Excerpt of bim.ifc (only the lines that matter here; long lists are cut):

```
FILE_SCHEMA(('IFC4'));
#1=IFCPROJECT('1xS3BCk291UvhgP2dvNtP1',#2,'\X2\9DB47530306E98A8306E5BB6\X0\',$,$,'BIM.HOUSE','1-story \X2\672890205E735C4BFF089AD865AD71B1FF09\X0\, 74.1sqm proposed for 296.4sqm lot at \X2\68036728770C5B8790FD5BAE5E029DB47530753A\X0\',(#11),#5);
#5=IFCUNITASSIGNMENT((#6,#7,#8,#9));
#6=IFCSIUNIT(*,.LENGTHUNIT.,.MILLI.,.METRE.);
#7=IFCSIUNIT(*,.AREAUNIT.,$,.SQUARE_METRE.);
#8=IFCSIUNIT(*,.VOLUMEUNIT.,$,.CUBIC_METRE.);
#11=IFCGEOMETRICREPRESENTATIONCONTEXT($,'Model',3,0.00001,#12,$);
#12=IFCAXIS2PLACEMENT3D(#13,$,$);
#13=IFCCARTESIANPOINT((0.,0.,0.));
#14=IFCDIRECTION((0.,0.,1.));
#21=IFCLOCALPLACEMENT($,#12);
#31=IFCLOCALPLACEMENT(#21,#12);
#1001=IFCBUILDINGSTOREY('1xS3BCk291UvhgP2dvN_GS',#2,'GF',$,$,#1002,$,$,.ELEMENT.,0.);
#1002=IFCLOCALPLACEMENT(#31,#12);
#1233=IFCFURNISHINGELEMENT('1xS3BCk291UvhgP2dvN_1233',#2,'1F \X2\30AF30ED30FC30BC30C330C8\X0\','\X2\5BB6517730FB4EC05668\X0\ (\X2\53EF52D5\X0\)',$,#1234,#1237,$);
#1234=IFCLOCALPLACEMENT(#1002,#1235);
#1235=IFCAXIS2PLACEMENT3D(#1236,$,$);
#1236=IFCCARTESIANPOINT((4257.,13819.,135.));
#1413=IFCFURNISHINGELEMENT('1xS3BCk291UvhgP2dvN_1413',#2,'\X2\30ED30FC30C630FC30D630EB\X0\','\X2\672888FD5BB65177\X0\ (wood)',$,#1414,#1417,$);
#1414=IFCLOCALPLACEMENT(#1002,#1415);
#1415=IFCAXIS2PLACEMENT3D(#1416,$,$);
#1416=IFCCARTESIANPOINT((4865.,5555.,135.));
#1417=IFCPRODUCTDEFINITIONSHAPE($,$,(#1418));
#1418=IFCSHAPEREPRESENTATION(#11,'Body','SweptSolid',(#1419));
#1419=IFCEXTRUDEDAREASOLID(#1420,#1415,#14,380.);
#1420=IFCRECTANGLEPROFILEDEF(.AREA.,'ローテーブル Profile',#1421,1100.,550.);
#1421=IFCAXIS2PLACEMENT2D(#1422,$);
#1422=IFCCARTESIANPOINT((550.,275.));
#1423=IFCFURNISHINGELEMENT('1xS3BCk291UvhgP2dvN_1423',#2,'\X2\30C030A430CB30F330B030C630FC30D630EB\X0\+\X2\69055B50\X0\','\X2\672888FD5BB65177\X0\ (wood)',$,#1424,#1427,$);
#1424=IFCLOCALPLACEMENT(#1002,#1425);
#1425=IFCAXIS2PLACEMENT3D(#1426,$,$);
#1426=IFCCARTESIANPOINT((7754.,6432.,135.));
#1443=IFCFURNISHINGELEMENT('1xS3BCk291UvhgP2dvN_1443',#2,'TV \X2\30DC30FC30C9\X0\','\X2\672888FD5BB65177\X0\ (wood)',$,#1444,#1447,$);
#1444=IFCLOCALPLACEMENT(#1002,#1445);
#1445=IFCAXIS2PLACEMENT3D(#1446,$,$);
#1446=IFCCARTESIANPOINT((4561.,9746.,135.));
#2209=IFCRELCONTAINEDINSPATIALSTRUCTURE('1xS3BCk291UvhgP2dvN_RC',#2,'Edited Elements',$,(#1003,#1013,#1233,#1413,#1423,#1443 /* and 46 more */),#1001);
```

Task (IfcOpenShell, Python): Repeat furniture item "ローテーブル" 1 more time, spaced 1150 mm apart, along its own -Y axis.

```python
import ifcopenshell
import ifcopenshell.api.geometry
import ifcopenshell.api.root
import ifcopenshell.util.element
import ifcopenshell.util.placement

model = ifcopenshell.open("bim.ifc")


def reuse_history(source, copy):
    """copy_class also copies each property set's owner history, people and application; keep the originals."""
    for rel in copy.IsDefinedBy:
        if rel.is_a("IfcRelDefinesByProperties") and (history := rel.RelatingPropertyDefinition.OwnerHistory):
            rel.RelatingPropertyDefinition.OwnerHistory = source.OwnerHistory
            ifcopenshell.util.element.remove_deep2(model, history)


source = model.by_id(1413)
base = ifcopenshell.util.placement.get_local_placement(source.ObjectPlacement)
step = -base[:3, 1] * 1150.0

for i in range(1, 2):
    copy = ifcopenshell.api.root.copy_class(model, product=source)
    copy.Representation = ifcopenshell.util.element.copy_deep(
        model, source.Representation, exclude=["IfcGeometricRepresentationContext", "IfcRepresentationMap"]
    )
    reuse_history(source, copy)
    matrix = base.copy()
    matrix[:3, 3] += i * step
    print("added at", matrix[:3, 3].round(3) + 0.0)
    ifcopenshell.api.geometry.edit_object_placement(model, product=copy, matrix=matrix, is_si=False)

model.write("bim_edited.ifc")
```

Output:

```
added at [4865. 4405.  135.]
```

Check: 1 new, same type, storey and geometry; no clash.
